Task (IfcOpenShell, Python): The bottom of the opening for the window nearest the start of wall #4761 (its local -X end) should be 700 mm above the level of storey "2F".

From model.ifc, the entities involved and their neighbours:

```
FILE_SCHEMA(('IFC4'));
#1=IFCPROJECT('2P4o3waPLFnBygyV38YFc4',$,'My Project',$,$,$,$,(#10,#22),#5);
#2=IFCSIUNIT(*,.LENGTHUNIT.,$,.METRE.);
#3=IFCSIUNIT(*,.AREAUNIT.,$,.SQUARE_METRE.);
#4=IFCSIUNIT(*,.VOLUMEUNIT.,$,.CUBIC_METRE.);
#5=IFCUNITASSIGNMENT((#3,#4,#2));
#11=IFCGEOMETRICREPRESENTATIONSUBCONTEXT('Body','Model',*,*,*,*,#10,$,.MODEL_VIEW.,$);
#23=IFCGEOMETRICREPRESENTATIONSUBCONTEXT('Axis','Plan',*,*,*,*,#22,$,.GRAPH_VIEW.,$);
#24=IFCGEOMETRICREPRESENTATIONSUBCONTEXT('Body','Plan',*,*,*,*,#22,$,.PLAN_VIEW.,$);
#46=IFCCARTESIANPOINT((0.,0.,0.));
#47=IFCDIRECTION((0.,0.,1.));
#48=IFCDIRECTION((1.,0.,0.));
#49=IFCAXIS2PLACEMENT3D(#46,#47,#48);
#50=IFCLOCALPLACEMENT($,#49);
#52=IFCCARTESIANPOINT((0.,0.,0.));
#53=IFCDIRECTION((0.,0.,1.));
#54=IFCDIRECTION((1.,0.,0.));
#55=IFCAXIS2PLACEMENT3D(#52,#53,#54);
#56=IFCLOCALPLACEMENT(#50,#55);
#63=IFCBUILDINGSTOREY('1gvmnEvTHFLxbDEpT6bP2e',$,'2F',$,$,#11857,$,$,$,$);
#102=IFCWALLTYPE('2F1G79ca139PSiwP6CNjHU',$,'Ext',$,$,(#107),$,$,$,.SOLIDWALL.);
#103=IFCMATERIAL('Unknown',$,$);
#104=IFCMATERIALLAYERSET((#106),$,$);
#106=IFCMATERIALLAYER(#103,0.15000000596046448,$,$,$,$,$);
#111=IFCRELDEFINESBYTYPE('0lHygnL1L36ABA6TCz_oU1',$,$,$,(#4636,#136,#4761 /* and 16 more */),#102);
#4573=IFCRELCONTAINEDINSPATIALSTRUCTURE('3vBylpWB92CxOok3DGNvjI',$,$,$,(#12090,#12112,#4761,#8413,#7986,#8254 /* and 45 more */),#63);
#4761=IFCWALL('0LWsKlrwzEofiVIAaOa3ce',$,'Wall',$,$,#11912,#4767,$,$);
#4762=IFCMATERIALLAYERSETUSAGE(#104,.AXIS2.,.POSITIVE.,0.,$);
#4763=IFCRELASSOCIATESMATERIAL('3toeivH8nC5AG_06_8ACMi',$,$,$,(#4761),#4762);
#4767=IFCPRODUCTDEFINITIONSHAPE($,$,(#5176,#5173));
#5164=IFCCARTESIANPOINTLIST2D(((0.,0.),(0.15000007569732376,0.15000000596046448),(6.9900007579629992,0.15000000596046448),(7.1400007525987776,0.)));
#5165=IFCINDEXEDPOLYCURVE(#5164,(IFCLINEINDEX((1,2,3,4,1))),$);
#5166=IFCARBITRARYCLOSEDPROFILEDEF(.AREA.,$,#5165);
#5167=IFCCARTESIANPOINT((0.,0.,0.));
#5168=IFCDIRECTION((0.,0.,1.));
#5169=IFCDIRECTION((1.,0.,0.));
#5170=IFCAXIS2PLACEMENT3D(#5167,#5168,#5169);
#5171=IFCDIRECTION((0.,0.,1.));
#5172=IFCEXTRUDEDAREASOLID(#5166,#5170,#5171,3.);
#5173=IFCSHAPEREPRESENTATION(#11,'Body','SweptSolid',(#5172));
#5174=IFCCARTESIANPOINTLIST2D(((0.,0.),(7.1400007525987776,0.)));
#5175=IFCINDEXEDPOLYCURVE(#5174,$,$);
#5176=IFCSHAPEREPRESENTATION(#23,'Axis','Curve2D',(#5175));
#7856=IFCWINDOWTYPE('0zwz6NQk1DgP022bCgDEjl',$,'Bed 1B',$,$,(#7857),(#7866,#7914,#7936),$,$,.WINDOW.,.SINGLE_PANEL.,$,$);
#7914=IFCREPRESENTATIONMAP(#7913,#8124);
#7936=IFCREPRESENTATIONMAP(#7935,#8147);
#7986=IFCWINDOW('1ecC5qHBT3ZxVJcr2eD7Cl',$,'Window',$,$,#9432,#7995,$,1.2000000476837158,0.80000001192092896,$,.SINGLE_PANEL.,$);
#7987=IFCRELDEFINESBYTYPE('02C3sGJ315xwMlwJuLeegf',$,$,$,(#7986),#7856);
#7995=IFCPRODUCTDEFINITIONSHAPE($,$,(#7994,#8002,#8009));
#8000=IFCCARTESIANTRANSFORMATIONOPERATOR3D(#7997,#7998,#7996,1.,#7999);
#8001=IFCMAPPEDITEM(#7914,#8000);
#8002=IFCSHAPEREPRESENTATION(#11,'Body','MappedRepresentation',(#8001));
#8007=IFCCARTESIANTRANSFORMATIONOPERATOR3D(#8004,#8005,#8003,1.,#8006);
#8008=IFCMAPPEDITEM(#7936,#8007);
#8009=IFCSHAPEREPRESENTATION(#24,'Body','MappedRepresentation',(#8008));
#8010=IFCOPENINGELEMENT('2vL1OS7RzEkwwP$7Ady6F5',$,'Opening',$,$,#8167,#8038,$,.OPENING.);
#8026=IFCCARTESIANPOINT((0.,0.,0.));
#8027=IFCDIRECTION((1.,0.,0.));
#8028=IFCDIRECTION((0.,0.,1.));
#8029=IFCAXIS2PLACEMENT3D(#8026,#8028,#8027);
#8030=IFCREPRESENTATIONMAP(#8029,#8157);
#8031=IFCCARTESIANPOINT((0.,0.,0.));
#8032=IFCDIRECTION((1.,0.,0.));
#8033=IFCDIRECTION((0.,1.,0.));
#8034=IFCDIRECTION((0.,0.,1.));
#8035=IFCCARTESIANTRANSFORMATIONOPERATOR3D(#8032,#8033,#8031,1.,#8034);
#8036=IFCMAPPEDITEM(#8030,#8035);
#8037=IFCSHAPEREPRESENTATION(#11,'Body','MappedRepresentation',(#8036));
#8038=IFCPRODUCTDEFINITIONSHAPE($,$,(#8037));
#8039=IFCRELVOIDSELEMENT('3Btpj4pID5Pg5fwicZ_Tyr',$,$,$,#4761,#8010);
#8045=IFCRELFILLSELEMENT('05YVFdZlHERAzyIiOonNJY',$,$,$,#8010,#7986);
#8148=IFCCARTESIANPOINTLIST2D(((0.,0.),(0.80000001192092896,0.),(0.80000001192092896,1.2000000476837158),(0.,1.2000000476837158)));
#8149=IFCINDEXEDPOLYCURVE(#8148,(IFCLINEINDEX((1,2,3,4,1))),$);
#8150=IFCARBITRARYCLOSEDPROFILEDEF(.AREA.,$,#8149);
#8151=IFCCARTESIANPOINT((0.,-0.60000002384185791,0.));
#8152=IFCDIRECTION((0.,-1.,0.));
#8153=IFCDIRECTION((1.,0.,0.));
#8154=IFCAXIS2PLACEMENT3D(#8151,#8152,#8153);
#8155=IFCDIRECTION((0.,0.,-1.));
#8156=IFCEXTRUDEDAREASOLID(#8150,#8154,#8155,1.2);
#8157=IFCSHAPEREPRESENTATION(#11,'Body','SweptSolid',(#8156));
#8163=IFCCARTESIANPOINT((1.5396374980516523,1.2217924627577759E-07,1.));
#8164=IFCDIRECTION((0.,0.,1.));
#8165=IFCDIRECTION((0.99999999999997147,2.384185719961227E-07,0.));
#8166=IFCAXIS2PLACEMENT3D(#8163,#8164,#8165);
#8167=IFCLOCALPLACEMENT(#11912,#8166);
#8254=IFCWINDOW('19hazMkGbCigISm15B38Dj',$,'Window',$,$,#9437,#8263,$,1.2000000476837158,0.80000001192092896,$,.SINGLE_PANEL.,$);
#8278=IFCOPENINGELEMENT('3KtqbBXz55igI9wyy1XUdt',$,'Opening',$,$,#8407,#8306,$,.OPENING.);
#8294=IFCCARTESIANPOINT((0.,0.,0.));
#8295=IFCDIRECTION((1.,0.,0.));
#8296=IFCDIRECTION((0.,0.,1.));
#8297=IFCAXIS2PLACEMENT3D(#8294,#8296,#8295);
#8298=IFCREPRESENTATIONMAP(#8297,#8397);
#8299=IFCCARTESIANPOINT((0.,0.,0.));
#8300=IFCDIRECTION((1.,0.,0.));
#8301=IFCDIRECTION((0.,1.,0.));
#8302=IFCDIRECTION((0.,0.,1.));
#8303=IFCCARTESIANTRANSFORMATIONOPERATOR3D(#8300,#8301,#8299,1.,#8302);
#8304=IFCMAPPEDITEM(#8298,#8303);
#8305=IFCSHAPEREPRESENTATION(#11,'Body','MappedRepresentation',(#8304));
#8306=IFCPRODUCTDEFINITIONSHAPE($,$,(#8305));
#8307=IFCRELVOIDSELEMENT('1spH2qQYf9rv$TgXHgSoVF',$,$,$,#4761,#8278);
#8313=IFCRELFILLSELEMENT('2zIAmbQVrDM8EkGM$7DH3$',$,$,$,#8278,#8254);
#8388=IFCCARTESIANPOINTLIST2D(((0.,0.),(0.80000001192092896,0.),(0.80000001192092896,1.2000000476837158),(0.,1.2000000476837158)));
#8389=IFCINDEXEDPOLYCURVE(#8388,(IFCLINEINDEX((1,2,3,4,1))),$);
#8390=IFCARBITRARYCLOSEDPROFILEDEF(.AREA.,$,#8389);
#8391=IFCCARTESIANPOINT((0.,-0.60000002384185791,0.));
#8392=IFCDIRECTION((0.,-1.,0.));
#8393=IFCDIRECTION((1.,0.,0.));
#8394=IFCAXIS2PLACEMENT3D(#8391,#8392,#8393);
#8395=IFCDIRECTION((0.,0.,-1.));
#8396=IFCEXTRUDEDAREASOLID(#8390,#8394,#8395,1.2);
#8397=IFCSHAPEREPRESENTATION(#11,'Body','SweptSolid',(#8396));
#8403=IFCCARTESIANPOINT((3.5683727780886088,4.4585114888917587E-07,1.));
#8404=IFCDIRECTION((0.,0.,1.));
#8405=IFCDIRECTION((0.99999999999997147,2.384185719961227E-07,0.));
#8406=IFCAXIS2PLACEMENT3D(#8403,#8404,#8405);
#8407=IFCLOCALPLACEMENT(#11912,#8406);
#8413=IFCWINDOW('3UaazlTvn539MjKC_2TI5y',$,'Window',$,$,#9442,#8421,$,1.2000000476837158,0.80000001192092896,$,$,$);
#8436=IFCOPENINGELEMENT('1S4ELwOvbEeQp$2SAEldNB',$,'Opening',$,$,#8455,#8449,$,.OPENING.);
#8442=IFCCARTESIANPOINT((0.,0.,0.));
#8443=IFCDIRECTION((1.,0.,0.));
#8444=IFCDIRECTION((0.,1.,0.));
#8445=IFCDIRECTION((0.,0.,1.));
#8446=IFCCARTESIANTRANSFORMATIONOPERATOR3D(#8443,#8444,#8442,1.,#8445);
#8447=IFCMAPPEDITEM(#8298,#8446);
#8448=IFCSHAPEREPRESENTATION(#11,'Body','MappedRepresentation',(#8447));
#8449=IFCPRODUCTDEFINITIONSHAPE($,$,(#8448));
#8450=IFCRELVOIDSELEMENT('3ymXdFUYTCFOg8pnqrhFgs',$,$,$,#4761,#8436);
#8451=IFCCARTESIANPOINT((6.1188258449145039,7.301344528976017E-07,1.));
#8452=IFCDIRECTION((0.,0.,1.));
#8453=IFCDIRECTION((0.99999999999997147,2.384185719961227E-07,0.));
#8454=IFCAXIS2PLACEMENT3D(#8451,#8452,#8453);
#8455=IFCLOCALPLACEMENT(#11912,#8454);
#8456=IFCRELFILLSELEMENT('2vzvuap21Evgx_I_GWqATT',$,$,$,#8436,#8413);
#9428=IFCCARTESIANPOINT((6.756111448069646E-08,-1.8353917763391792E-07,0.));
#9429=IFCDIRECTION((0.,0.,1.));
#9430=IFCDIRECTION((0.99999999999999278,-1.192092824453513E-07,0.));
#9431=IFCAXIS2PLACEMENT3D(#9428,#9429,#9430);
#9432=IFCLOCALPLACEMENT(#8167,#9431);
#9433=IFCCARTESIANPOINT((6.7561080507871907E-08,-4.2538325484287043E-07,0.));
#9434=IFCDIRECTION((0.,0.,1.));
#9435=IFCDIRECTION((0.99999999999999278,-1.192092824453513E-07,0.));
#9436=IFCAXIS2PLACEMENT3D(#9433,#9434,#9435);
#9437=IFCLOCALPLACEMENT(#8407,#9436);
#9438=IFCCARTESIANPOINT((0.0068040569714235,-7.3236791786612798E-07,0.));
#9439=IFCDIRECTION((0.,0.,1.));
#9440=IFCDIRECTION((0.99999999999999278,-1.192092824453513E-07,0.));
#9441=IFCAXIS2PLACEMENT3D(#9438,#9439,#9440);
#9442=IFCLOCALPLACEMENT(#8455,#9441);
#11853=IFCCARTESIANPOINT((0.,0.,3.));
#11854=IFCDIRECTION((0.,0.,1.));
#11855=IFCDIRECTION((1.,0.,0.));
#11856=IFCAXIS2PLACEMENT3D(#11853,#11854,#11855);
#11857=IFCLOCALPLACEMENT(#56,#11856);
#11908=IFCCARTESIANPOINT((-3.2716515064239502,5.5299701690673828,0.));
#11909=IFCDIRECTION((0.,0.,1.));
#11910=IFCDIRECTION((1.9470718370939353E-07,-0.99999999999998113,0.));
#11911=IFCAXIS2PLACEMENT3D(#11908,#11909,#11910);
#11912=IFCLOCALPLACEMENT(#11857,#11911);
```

```python
import numpy as np
import ifcopenshell
import ifcopenshell.api.geometry
import ifcopenshell.geom
import ifcopenshell.util.element
import ifcopenshell.util.placement
import ifcopenshell.util.shape
import ifcopenshell.util.unit

model = ifcopenshell.open("model.ifc")
unit_scale = ifcopenshell.util.unit.calculate_unit_scale(model)

window = model.by_guid("1ecC5qHBT3ZxVJcr2eD7Cl")
opening = window.FillsVoids[0].RelatingOpeningElement
storey = ifcopenshell.util.element.get_container(window, ifc_class="IfcBuildingStorey")
level = ifcopenshell.util.placement.get_local_placement(storey.ObjectPlacement)[2, 3]

# The opening's origin need not be at the sill, so measure its lowest point.
shape = ifcopenshell.geom.create_shape(ifcopenshell.geom.settings(), opening)
bottom = ifcopenshell.util.shape.get_shape_bottom_elevation(shape, shape.geometry) / unit_scale
dz = level + 0.7 / unit_scale - bottom

shift = np.array([0.0, 0.0, dz])
# The window is placed relative to its opening, so it follows when the opening moves.
matrix = ifcopenshell.util.placement.get_local_placement(opening.ObjectPlacement)
matrix[:3, 3] += shift
ifcopenshell.api.geometry.edit_object_placement(
    model, product=opening, matrix=matrix, is_si=False, should_transform_children=True
)

print(f"moved by {dz * unit_scale:+.3f} m")

model.write("model-out.ifc")
```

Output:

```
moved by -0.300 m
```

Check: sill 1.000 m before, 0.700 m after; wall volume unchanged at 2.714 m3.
